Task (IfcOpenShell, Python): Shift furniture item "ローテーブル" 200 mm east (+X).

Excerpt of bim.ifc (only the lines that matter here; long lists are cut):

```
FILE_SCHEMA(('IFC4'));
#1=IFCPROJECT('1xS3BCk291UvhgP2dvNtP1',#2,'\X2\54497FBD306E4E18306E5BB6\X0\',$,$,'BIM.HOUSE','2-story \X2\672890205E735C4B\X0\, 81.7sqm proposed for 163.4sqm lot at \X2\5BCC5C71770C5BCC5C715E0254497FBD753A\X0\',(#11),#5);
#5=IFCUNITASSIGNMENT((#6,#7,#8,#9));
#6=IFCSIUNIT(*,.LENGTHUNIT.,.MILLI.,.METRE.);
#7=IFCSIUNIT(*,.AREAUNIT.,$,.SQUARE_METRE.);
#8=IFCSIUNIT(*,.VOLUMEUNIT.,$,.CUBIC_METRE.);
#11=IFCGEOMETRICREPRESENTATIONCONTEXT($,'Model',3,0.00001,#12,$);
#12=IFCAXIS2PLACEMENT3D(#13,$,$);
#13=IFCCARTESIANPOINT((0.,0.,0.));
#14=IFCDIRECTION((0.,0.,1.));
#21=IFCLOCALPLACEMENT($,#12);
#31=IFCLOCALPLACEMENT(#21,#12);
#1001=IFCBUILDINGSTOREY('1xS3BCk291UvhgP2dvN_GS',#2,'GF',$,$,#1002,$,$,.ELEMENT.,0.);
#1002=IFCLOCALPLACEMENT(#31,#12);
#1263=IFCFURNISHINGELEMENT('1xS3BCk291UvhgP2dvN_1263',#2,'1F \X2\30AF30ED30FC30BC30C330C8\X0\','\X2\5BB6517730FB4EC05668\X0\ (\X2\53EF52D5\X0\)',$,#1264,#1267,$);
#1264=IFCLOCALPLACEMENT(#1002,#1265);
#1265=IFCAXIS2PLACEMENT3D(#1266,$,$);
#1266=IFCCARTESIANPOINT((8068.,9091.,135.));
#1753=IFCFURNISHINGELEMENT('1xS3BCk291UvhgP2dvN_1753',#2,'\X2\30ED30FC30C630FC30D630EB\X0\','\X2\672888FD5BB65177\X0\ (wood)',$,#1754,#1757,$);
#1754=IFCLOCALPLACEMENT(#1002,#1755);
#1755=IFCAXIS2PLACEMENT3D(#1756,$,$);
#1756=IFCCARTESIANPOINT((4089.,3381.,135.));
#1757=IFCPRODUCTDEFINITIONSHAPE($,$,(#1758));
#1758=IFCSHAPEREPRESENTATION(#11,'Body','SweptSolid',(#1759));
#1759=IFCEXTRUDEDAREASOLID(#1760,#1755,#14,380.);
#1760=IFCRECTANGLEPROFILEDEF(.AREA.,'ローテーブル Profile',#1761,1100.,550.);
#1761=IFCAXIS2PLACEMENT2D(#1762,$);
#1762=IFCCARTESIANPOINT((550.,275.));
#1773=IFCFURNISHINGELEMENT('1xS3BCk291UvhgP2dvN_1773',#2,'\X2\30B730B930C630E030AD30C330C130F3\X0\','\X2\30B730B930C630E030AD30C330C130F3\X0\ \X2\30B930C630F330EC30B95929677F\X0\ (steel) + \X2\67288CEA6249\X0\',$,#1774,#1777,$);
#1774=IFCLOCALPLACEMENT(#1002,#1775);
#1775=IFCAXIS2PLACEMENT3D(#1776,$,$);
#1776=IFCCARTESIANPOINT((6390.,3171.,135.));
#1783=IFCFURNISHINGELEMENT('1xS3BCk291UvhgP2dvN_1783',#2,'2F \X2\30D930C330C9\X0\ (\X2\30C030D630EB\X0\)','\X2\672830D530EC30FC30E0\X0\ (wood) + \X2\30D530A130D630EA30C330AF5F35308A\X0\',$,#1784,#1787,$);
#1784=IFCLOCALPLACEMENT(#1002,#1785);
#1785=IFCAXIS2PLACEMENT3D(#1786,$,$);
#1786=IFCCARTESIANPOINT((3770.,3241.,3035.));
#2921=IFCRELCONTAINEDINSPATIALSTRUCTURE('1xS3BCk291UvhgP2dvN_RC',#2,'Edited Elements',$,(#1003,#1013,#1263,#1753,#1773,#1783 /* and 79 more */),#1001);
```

```python
import ifcopenshell
import ifcopenshell.api.geometry
import ifcopenshell.util.placement
import ifcopenshell.util.unit

model = ifcopenshell.open("bim.ifc")
unit_scale = ifcopenshell.util.unit.calculate_unit_scale(model)

item = model.by_guid("1xS3BCk291UvhgP2dvN_1753")
matrix = ifcopenshell.util.placement.get_local_placement(item.ObjectPlacement)
matrix[0, 3] += 0.2 / unit_scale
ifcopenshell.api.geometry.edit_object_placement(model, product=item, matrix=matrix, is_si=False)

print(ifcopenshell.util.placement.get_local_placement(item.ObjectPlacement).round(3) + 0.0)

model.write("bim_rev.ifc")
```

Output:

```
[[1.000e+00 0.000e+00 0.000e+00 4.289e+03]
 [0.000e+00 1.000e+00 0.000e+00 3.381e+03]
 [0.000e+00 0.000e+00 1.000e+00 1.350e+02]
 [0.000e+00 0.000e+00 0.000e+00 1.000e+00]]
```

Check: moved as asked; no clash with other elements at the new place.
